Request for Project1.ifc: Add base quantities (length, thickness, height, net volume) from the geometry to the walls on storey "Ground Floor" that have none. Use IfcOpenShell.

First a look at what the model holds.

```python
import ifcopenshell
import ifcopenshell.util.element
import ifcopenshell.util.unit

model = ifcopenshell.open("Project1.ifc")
print(model.schema)
for unit_type in ("LENGTHUNIT", "AREAUNIT", "VOLUMEUNIT"):
    print(unit_type, ifcopenshell.util.unit.calculate_unit_scale(model, unit_type))
storey = next(s for s in model.by_type("IfcBuildingStorey") if s.Name == "Ground Floor")
walls = [e for e in ifcopenshell.util.element.get_decomposition(storey) if e.is_a("IfcWall")]
for e in sorted(walls, key=lambda e: e.id()):
    print(e.id(), e.is_a(), e.Name, list(ifcopenshell.util.element.get_psets(e, qtos_only=True)), sep=" | ")
```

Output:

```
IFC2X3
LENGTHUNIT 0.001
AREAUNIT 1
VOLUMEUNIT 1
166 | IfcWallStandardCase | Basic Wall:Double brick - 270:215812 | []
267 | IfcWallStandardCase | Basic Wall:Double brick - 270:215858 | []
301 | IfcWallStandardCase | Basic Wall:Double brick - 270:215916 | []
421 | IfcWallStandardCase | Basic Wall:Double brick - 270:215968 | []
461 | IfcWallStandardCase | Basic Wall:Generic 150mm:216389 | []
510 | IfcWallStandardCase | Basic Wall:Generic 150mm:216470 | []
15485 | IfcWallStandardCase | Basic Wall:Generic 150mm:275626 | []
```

```python
import ifcopenshell
import ifcopenshell.api.pset
import ifcopenshell.geom
import ifcopenshell.util.element
import ifcopenshell.util.shape
import ifcopenshell.util.unit

model = ifcopenshell.open("Project1.ifc")
unit_scale = ifcopenshell.util.unit.calculate_unit_scale(model)
volume_scale = ifcopenshell.util.unit.calculate_unit_scale(model, "VOLUMEUNIT")
settings = ifcopenshell.geom.settings()

storey = next(s for s in model.by_type("IfcBuildingStorey") if s.Name == "Ground Floor")
walls = [e for e in ifcopenshell.util.element.get_decomposition(storey) if e.is_a("IfcWall")]

for e in sorted(walls, key=lambda e: e.id()):
    if ifcopenshell.util.element.get_psets(e, qtos_only=True, should_inherit=False):
        continue
    # Geometry comes back in metres, in the element's own axes.
    shape = ifcopenshell.geom.create_shape(settings, e)
    values = {
        "Length": ifcopenshell.util.shape.get_x(shape.geometry) / unit_scale,
        "Width": ifcopenshell.util.shape.get_y(shape.geometry) / unit_scale,
        "Height": ifcopenshell.util.shape.get_z(shape.geometry) / unit_scale,
        "NetVolume": ifcopenshell.util.shape.get_volume(shape.geometry) / volume_scale,
    }
    qto = ifcopenshell.api.pset.add_qto(model, product=e, name="BaseQuantities")
    ifcopenshell.api.pset.edit_qto(model, qto=qto, properties=values)
    print(e.id(), {k: round(v, 3) for k, v in values.items()})

model.write("Project1-out.ifc")
```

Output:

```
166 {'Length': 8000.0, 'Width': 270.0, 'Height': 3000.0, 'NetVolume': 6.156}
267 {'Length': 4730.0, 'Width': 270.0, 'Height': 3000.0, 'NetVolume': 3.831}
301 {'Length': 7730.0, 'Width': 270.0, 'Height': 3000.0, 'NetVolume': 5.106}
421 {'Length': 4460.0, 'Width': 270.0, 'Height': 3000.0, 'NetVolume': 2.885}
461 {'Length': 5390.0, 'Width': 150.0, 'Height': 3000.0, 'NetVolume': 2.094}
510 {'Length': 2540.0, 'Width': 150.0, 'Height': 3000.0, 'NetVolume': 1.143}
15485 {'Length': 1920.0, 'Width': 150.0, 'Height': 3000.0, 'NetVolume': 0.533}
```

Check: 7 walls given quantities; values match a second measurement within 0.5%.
